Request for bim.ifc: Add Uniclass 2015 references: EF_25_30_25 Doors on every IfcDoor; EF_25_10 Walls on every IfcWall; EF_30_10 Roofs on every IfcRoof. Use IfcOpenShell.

First a look at what the model holds.

```python
import ifcopenshell

model = ifcopenshell.open("bim.ifc")
print(model.schema)
print("classifications:", [c.Name for c in model.by_type("IfcClassification")])
for ifc_class in ("IfcDoor", "IfcRoof", "IfcStair", "IfcWall", "IfcWindow"):
    print(ifc_class, len(model.by_type(ifc_class)))
```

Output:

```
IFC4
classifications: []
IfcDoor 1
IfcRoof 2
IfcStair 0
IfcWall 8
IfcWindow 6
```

```python
import ifcopenshell
import ifcopenshell.api.classification

model = ifcopenshell.open("bim.ifc")

system = ifcopenshell.api.classification.add_classification(model, classification="Uniclass 2015")

codes = {
    "IfcDoor": ("EF_25_30_25", "Doors"),
    "IfcWall": ("EF_25_10", "Walls"),
    "IfcRoof": ("EF_30_10", "Roofs"),
}
for ifc_class, (code, name) in codes.items():
    products = model.by_type(ifc_class)
    ifcopenshell.api.classification.add_reference(
        model, products=products, classification=system, identification=code, name=name
    )
    print(code, len(products))

model.write("bim_rev.ifc")
```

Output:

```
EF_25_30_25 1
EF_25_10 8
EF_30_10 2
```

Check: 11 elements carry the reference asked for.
